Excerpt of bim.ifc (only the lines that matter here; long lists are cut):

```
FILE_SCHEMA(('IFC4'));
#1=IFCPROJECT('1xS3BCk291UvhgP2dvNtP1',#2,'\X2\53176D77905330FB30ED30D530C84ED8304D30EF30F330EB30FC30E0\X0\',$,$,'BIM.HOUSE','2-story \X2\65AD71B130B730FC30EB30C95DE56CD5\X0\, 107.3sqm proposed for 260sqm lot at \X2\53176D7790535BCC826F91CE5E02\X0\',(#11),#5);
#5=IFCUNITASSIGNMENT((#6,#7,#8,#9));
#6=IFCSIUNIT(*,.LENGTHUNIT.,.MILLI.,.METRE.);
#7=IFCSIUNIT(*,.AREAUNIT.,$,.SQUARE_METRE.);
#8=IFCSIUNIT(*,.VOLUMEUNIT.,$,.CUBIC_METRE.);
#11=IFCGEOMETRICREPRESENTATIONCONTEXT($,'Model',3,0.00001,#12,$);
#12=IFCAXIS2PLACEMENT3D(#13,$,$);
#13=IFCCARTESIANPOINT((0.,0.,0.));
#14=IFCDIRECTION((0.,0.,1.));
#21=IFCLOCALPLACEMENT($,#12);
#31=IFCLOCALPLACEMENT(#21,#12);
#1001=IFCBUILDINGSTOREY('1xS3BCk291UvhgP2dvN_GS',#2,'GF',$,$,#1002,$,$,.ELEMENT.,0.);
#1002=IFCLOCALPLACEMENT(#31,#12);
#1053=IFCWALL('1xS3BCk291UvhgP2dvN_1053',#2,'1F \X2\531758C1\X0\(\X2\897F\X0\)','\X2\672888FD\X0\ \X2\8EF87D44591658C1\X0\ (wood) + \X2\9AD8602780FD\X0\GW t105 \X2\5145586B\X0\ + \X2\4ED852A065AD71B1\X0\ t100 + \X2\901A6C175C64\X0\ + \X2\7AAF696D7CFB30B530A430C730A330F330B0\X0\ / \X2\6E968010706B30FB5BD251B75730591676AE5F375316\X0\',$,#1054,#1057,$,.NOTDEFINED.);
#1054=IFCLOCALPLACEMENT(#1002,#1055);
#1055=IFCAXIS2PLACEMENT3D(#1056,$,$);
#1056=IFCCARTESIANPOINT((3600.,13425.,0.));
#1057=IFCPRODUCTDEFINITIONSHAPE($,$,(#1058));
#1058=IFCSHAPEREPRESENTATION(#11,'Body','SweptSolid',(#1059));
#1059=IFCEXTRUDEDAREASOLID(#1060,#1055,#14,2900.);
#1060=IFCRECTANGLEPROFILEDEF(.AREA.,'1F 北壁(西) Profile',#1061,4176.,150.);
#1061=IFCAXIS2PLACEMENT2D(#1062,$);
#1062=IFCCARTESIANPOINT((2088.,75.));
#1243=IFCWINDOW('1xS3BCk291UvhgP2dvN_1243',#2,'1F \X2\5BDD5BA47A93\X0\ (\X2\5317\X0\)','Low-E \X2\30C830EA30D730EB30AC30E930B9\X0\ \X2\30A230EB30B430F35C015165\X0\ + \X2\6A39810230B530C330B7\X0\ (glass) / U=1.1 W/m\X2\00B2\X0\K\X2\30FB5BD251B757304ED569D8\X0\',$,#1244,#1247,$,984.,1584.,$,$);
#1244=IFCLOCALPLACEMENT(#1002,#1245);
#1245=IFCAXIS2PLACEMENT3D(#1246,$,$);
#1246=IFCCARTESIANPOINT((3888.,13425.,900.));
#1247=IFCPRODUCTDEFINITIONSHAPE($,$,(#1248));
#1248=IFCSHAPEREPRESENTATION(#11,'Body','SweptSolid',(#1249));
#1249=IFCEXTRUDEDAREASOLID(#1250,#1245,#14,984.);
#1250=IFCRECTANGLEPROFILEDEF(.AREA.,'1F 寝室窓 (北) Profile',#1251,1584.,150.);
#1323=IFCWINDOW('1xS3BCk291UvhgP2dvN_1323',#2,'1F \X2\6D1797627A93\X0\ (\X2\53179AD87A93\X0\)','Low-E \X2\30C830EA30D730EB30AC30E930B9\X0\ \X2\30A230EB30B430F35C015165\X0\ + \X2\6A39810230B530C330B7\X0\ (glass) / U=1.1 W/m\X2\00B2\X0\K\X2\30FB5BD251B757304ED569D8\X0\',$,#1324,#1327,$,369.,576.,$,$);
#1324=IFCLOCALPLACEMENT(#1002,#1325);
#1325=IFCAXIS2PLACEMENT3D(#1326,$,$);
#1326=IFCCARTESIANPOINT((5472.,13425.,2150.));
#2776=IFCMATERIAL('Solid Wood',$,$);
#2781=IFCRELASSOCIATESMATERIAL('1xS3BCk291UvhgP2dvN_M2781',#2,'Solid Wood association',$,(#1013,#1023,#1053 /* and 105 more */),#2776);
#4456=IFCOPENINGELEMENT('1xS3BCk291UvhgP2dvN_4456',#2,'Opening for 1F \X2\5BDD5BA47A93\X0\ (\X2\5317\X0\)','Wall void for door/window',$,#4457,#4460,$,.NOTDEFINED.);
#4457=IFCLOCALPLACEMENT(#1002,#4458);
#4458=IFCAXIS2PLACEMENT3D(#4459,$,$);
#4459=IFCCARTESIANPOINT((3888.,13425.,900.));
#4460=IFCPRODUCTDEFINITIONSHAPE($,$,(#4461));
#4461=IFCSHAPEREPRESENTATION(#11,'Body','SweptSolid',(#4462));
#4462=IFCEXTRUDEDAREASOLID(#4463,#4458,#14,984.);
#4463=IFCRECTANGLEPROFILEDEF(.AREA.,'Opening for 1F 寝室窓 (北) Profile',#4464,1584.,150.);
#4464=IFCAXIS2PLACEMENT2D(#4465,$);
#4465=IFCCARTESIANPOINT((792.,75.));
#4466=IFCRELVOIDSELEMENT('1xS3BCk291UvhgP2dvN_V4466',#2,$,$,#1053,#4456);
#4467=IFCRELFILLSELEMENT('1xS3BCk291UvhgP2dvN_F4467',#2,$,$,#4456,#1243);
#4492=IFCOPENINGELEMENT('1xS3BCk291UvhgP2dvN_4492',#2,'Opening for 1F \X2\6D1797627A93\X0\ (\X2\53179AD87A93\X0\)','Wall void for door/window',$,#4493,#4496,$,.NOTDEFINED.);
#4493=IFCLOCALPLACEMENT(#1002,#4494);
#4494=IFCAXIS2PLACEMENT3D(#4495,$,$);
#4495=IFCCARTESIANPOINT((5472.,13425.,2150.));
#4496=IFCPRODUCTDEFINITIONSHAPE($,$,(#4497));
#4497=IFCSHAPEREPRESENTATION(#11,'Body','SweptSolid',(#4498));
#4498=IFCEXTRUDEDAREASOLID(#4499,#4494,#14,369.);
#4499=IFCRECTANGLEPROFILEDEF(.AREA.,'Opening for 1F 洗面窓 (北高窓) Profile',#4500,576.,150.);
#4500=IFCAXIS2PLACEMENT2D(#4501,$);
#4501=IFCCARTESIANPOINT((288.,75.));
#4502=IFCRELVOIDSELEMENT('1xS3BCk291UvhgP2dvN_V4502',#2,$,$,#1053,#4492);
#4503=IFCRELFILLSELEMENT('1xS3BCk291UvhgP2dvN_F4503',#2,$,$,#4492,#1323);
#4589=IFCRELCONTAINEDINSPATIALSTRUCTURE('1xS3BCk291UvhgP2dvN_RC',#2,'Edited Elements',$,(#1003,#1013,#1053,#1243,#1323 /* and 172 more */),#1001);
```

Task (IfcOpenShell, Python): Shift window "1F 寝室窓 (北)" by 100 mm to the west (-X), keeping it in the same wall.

```python
import ifcopenshell
import ifcopenshell.api.geometry
import ifcopenshell.util.placement
import ifcopenshell.util.unit

model = ifcopenshell.open("bim.ifc")
unit_scale = ifcopenshell.util.unit.calculate_unit_scale(model)

window = model.by_guid("1xS3BCk291UvhgP2dvN_1243")
opening = window.FillsVoids[0].RelatingOpeningElement
wall = opening.VoidsElements[0].RelatingBuildingElement

wall_matrix = ifcopenshell.util.placement.get_local_placement(wall.ObjectPlacement)
shift = wall_matrix[:3, 0] * -0.1 / unit_scale
before = ifcopenshell.util.placement.get_local_placement(window.ObjectPlacement)[:3, 3].copy()

# The window is not placed relative to its opening, so move both.
for product in (opening, window):
    matrix = ifcopenshell.util.placement.get_local_placement(product.ObjectPlacement)
    matrix[:3, 3] += shift
    ifcopenshell.api.geometry.edit_object_placement(model, product=product, matrix=matrix, is_si=False)

after = ifcopenshell.util.placement.get_local_placement(window.ObjectPlacement)[:3, 3]
print("window moved by", (after - before).round(3) + 0.0)

model.write("bim_updated.ifc")
```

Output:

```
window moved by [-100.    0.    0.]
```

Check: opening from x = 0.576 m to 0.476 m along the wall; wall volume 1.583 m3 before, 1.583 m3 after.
